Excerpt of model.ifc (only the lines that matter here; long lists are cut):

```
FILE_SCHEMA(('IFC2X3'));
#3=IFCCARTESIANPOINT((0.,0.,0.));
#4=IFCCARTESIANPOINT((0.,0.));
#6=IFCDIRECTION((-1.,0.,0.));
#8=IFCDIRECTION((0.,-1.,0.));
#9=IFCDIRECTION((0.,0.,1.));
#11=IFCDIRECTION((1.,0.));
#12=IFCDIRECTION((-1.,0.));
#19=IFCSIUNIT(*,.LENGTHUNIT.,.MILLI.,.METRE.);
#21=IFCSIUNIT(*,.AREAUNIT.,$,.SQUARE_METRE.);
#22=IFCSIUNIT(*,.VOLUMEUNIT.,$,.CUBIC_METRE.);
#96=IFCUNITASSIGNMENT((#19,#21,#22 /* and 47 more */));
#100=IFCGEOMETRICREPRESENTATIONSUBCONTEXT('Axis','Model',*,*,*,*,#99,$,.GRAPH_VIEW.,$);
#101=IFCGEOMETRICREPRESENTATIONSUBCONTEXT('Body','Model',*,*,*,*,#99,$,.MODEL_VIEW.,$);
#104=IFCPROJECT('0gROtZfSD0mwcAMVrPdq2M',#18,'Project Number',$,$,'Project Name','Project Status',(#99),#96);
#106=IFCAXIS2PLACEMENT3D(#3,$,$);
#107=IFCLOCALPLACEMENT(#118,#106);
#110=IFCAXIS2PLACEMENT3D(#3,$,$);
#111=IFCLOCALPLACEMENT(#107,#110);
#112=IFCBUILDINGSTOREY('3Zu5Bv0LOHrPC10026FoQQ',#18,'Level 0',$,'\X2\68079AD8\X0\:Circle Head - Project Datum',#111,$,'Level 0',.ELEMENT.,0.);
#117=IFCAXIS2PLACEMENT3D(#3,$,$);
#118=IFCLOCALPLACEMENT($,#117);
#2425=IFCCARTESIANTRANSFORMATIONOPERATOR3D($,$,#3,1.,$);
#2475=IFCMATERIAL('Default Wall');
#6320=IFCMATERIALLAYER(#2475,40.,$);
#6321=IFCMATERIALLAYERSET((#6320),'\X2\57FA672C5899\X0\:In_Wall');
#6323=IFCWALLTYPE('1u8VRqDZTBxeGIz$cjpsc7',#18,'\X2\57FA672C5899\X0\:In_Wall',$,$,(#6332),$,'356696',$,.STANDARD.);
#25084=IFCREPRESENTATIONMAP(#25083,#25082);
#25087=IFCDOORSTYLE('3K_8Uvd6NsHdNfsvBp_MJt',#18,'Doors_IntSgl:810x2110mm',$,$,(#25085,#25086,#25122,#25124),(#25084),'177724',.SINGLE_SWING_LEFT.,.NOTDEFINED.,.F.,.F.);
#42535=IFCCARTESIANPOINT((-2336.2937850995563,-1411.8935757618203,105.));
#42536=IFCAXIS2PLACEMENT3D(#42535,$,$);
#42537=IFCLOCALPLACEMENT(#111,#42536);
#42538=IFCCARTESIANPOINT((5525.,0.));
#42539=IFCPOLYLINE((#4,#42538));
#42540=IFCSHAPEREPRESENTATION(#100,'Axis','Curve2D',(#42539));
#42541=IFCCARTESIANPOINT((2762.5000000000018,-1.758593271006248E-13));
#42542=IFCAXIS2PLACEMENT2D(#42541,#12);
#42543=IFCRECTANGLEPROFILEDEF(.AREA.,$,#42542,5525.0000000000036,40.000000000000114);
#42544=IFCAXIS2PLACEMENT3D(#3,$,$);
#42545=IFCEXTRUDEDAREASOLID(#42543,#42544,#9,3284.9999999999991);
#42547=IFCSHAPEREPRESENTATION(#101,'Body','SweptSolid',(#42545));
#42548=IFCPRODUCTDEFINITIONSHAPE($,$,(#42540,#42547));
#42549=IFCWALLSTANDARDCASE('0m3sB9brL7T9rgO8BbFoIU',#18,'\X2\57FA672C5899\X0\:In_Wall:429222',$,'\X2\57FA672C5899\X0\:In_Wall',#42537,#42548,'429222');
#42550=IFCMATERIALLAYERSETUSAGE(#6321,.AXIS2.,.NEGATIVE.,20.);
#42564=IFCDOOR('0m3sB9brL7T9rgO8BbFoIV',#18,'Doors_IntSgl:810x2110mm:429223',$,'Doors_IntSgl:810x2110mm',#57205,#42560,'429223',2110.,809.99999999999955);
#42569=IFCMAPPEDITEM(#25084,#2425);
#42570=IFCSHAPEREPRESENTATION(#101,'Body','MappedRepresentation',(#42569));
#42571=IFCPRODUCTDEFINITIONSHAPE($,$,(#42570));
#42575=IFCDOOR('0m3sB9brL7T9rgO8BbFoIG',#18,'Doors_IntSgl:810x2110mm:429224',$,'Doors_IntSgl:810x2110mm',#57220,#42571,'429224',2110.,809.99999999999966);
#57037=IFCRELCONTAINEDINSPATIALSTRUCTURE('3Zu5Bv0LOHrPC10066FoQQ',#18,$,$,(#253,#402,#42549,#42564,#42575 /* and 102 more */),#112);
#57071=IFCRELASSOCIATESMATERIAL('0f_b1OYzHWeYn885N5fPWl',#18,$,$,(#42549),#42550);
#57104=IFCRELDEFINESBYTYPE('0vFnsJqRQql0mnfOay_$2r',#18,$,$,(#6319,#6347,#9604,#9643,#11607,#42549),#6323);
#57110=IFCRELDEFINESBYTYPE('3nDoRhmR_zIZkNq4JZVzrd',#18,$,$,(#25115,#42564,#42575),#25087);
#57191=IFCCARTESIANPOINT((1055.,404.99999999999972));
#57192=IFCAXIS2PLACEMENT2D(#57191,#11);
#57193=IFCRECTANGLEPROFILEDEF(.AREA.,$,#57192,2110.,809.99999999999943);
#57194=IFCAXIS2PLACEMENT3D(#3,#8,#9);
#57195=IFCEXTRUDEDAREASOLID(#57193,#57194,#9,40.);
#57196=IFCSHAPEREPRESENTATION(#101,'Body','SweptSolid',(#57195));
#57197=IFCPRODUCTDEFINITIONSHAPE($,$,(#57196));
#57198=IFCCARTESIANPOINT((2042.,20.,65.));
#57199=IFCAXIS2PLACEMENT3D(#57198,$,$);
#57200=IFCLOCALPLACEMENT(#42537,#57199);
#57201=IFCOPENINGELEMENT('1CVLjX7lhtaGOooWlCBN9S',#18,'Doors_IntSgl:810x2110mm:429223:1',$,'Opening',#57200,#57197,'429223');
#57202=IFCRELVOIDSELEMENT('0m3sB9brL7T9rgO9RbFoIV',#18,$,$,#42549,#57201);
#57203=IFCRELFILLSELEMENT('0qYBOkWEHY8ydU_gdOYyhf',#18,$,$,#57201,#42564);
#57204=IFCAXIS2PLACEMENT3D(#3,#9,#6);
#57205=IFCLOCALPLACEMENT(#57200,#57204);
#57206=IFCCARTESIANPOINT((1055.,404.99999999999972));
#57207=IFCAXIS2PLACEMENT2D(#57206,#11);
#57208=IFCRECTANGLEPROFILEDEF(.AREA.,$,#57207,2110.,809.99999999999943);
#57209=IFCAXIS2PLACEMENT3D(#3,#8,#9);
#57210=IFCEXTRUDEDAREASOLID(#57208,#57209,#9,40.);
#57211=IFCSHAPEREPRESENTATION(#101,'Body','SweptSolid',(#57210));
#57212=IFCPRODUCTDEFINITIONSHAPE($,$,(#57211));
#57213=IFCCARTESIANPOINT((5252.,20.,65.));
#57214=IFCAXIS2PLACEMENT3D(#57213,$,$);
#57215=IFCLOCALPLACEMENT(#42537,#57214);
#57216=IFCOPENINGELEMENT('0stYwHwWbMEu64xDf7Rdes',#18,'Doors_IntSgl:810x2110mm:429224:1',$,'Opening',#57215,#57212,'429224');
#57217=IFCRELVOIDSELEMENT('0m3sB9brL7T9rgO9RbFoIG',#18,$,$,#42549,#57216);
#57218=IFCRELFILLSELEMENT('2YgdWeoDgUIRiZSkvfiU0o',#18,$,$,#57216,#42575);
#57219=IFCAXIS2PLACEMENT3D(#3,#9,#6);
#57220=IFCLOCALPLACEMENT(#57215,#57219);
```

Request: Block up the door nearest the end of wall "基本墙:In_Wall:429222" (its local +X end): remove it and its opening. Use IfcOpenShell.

```python
import ifcopenshell
import ifcopenshell.api.feature
import ifcopenshell.api.root
import ifcopenshell.geom
import ifcopenshell.util.shape

model = ifcopenshell.open("model.ifc")
settings = ifcopenshell.geom.settings()


def volume(element):
    """Net volume in cubic metres, openings subtracted."""
    shape = ifcopenshell.geom.create_shape(settings, element)
    return ifcopenshell.util.shape.get_volume(shape.geometry)


door = model.by_guid("0m3sB9brL7T9rgO8BbFoIG")
opening = door.FillsVoids[0].RelatingOpeningElement
wall = opening.VoidsElements[0].RelatingBuildingElement
before = volume(wall)

ifcopenshell.api.root.remove_product(model, product=door)
ifcopenshell.api.feature.remove_feature(model, feature=opening)

after = volume(wall)

print(f"wall volume {before:.3f} -> {after:.3f} m3")

model.write("model_v2.ifc")
```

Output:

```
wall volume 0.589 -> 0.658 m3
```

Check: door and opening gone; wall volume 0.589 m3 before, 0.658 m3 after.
